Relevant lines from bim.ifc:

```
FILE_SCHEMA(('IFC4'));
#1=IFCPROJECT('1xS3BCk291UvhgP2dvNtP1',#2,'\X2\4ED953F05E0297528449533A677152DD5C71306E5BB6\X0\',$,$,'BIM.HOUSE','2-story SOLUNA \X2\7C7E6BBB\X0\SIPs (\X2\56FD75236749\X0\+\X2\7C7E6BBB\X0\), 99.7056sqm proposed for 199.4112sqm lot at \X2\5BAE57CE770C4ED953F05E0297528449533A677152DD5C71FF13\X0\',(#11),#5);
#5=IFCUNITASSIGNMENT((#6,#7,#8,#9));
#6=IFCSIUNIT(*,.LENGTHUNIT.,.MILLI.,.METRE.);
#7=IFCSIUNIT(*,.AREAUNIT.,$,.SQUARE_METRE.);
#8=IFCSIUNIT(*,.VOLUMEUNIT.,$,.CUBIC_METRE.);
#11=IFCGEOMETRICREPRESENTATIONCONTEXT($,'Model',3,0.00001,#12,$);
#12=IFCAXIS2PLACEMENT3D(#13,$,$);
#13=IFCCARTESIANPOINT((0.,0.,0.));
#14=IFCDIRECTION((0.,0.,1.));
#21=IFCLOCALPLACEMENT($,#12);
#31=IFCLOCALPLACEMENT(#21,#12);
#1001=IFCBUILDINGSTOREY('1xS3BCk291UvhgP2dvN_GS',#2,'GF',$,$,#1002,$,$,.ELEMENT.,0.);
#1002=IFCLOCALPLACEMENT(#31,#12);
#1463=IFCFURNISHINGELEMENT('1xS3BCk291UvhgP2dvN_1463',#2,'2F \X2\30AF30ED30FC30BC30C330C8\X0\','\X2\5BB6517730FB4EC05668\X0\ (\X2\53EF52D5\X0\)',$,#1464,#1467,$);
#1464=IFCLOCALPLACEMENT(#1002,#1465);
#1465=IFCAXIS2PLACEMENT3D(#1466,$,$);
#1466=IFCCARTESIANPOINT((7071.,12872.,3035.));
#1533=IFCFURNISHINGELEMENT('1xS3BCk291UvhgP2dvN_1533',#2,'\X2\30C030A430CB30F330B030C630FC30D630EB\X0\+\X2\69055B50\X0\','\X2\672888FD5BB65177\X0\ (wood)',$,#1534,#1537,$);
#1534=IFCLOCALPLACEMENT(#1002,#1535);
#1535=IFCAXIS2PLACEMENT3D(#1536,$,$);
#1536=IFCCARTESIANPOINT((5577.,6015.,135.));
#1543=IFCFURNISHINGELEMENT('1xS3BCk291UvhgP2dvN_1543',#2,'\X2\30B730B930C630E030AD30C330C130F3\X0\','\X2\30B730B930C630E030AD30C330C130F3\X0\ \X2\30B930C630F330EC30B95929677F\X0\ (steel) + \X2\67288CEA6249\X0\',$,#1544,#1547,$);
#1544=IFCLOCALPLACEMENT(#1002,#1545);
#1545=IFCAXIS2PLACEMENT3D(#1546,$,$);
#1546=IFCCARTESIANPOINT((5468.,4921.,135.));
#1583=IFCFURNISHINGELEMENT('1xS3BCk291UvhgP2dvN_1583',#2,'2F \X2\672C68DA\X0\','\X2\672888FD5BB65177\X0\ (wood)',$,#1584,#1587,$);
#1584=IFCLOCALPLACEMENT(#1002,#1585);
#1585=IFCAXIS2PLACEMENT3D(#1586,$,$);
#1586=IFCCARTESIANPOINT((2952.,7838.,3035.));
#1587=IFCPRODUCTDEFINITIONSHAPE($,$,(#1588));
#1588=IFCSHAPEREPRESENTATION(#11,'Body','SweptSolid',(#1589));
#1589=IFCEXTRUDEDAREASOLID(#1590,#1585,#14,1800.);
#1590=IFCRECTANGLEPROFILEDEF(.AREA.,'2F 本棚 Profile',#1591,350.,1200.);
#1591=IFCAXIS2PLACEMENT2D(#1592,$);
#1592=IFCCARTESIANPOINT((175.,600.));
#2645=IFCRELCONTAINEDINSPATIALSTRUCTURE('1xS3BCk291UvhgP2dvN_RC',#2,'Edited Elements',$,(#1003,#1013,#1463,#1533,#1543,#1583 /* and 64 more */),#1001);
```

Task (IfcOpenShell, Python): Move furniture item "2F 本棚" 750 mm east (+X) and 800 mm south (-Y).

```python
import ifcopenshell
import ifcopenshell.api.geometry
import ifcopenshell.util.placement
import ifcopenshell.util.unit

model = ifcopenshell.open("bim.ifc")
unit_scale = ifcopenshell.util.unit.calculate_unit_scale(model)

item = model.by_guid("1xS3BCk291UvhgP2dvN_1583")
matrix = ifcopenshell.util.placement.get_local_placement(item.ObjectPlacement)
matrix[0, 3] += 0.75 / unit_scale
matrix[1, 3] -= 0.8 / unit_scale
ifcopenshell.api.geometry.edit_object_placement(model, product=item, matrix=matrix, is_si=False)

print(ifcopenshell.util.placement.get_local_placement(item.ObjectPlacement).round(3) + 0.0)

model.write("bim_edited.ifc")
```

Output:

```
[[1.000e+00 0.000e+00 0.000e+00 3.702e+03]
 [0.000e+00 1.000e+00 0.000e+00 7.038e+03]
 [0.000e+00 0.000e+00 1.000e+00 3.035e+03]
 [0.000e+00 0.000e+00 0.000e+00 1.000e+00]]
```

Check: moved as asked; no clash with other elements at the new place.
